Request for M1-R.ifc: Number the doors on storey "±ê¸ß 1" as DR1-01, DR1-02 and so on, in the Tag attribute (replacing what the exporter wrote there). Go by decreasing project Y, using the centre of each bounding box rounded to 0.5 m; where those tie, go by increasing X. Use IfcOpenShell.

First a look at what the model holds.

```python
import ifcopenshell
import ifcopenshell.util.element
import ifcopenshell.util.placement

model = ifcopenshell.open("M1-R.ifc")
print(model.schema)
storey = next(s for s in model.by_type("IfcBuildingStorey") if s.Name == "±ê¸ß 1")
doors = [e for e in ifcopenshell.util.element.get_decomposition(storey) if e.is_a("IfcDoor")]
for e in sorted(doors, key=lambda e: e.id()):
    origin = ifcopenshell.util.placement.get_local_placement(e.ObjectPlacement)[:3, 3]
    print(e.id(), e.Tag, e.Name, origin.round(2) + 0.0, sep=" | ")
```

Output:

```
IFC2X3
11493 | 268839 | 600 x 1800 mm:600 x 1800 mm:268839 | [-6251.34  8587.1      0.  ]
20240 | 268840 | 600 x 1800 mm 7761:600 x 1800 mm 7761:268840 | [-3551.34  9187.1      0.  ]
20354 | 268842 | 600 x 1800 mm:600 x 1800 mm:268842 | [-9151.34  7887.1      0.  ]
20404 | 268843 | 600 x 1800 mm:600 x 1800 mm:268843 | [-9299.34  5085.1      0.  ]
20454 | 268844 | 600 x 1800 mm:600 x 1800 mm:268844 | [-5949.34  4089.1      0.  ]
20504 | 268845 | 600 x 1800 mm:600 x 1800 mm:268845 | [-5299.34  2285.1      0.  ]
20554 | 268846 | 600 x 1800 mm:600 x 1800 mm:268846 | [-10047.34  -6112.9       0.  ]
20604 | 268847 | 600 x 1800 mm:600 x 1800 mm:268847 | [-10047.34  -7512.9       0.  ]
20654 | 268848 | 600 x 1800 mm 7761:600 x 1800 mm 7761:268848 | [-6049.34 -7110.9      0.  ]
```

```python
import ifcopenshell
import ifcopenshell.geom
import ifcopenshell.util.element
import ifcopenshell.util.shape

model = ifcopenshell.open("M1-R.ifc")
settings = ifcopenshell.geom.settings()
settings.set("use-world-coords", True)


def centre(element):
    shape = ifcopenshell.geom.create_shape(settings, element)
    return ifcopenshell.util.shape.get_bbox_centroid(shape.geometry)


storey = next(s for s in model.by_type("IfcBuildingStorey") if s.Name == "±ê¸ß 1")
doors = [e for e in ifcopenshell.util.element.get_decomposition(storey) if e.is_a("IfcDoor")]

# Insertion points can sit at a corner or the storey origin, so sort by the geometry (in metres).
centres = {e: centre(e) for e in doors}
doors.sort(key=lambda e: (-round(centres[e][1] / 0.5), centres[e][0]))

for i, e in enumerate(doors, start=1):
    number = f"DR1-{i:02d}"
    e.Tag = number
    print(e.id(), number)

model.write("M1-R-out.ifc")
```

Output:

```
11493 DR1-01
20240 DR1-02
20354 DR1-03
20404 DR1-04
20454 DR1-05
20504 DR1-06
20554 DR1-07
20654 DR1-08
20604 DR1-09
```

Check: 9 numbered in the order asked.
